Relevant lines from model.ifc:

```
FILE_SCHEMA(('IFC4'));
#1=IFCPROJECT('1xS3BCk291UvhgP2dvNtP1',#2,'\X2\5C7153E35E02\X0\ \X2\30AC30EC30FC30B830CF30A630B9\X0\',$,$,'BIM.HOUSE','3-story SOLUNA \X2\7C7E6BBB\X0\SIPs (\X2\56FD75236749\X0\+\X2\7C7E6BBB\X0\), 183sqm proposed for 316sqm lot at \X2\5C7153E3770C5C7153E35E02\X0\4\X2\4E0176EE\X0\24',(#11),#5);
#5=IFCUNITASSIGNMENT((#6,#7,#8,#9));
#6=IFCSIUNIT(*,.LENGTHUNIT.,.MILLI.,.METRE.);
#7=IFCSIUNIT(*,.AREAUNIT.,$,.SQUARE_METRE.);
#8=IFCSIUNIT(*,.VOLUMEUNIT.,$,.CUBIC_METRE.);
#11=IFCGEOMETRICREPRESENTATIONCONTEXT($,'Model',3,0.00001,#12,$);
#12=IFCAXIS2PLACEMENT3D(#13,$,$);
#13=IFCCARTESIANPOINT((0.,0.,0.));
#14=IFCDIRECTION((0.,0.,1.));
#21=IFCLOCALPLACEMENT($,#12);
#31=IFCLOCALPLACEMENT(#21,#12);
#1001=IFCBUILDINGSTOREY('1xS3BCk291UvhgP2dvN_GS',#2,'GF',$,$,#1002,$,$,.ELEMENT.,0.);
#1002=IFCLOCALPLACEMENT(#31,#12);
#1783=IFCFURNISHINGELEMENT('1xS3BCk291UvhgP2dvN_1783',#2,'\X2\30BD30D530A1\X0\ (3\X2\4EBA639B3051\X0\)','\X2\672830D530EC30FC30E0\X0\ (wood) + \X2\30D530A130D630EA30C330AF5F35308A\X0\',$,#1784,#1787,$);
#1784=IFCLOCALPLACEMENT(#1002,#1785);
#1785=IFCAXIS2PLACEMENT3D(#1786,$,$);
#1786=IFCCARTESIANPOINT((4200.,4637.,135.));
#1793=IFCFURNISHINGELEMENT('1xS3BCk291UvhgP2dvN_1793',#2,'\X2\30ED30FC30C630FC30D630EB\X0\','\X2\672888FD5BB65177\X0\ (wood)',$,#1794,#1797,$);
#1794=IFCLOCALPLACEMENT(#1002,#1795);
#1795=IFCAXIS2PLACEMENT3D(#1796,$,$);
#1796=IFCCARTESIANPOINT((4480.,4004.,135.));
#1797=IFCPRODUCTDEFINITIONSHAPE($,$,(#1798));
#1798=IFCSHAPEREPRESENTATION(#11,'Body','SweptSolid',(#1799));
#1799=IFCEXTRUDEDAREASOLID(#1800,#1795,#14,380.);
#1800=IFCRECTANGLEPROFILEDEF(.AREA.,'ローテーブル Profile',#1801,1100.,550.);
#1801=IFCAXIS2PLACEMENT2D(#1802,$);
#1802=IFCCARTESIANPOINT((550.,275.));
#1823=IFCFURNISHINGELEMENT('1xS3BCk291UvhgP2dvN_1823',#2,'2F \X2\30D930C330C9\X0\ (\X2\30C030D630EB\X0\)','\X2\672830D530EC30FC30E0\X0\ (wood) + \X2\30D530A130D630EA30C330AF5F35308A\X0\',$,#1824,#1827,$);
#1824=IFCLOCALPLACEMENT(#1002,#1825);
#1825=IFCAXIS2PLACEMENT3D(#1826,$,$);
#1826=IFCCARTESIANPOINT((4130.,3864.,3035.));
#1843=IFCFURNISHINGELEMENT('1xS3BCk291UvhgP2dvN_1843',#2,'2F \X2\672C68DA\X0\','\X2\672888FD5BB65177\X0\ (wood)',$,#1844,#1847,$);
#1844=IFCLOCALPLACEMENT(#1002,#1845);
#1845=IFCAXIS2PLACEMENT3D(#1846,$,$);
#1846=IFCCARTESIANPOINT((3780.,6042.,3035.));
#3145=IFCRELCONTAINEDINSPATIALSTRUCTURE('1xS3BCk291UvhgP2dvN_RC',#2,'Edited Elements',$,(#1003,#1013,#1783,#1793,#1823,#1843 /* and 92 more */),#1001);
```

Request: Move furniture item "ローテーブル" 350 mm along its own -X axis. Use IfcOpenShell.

```python
import ifcopenshell
import ifcopenshell.api.geometry
import ifcopenshell.util.placement
import ifcopenshell.util.unit

model = ifcopenshell.open("model.ifc")
unit_scale = ifcopenshell.util.unit.calculate_unit_scale(model)

item = model.by_id(1793)
matrix = ifcopenshell.util.placement.get_local_placement(item.ObjectPlacement)
matrix[:3, 3] -= matrix[:3, 0] * 0.35 / unit_scale
ifcopenshell.api.geometry.edit_object_placement(model, product=item, matrix=matrix, is_si=False)

print(ifcopenshell.util.placement.get_local_placement(item.ObjectPlacement).round(3) + 0.0)

model.write("model_rev.ifc")
```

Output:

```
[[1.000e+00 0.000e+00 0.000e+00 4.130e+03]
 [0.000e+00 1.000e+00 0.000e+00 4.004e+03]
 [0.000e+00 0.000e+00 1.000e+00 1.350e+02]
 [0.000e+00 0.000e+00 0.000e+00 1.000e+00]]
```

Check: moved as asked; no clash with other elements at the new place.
